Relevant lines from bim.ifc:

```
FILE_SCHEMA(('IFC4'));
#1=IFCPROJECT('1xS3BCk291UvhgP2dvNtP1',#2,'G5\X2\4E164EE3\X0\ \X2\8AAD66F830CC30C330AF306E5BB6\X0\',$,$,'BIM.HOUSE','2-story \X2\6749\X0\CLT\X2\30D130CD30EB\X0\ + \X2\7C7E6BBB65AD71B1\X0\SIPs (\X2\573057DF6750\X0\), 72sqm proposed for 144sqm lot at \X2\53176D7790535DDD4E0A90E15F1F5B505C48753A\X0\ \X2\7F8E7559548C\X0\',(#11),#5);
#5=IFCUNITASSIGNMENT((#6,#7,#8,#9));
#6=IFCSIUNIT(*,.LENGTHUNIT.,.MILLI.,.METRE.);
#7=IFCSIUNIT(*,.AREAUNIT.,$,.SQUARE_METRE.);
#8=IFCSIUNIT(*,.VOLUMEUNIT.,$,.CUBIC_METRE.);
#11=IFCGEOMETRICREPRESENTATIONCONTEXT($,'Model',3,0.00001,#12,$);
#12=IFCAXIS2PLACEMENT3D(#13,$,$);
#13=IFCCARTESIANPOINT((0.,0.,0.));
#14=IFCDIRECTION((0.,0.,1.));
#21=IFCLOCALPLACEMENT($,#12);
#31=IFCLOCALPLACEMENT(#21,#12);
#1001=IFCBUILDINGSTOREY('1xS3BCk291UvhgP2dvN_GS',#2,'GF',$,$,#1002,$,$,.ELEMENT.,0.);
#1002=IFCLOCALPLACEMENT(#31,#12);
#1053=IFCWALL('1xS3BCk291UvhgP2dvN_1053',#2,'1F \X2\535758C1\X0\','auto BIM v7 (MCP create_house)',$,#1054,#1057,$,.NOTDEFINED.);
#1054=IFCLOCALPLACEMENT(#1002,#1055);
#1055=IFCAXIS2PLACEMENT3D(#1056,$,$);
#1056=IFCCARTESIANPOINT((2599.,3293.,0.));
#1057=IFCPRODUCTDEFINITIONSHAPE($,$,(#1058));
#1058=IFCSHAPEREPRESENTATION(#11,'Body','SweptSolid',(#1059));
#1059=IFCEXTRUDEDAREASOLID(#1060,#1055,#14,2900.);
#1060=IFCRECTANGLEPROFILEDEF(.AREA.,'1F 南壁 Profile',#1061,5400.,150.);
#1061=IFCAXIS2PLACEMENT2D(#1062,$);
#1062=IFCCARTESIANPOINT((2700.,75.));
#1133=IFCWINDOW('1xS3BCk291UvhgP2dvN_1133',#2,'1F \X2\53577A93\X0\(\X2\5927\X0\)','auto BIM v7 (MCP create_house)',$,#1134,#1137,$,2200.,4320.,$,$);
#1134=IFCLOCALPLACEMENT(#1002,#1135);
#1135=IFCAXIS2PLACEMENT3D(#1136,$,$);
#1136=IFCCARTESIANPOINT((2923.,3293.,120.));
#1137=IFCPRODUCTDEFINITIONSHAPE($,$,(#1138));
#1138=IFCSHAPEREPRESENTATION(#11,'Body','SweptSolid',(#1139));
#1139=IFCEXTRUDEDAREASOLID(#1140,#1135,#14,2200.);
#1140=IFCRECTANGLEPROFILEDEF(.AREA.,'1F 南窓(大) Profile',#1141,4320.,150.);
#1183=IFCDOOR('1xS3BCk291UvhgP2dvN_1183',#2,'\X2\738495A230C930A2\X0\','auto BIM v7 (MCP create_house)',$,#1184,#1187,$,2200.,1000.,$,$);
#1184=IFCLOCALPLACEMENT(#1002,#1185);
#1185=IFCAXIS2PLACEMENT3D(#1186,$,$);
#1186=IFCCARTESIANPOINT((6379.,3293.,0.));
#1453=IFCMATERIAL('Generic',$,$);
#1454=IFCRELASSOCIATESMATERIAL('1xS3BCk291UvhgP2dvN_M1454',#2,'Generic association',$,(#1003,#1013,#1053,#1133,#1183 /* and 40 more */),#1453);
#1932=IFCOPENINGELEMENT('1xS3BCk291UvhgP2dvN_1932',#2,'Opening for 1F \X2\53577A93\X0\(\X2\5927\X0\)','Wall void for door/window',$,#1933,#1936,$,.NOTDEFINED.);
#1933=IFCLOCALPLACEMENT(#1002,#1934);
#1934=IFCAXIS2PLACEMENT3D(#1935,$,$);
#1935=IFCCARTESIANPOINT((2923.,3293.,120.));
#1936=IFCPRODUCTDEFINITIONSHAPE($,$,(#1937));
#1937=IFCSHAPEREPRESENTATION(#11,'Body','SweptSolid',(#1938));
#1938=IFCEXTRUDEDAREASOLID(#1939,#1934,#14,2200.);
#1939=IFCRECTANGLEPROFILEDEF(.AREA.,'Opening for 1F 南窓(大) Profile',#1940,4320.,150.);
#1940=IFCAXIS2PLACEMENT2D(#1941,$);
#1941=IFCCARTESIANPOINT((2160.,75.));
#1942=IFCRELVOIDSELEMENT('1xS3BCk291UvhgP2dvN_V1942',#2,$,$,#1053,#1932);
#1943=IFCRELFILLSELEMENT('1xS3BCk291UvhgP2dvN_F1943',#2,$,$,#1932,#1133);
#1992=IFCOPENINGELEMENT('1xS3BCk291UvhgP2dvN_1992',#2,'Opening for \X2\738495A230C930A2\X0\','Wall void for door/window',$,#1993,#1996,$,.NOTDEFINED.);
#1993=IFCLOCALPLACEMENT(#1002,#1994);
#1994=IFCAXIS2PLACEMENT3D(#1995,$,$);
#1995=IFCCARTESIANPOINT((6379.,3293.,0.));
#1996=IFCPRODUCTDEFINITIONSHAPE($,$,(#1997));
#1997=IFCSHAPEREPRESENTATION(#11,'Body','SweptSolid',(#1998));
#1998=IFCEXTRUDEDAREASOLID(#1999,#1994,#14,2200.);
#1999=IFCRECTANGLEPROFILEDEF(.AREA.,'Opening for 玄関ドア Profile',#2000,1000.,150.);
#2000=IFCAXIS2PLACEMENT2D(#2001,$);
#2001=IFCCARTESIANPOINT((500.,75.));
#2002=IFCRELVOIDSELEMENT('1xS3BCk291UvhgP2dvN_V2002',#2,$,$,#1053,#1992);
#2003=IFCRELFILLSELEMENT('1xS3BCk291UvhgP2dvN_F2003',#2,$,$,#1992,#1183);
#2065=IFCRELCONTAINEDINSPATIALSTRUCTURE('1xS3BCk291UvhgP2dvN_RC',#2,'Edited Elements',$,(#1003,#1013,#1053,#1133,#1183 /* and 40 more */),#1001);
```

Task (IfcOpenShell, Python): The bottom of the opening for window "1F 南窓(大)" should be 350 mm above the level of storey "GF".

```python
import numpy as np
import ifcopenshell
import ifcopenshell.api.geometry
import ifcopenshell.geom
import ifcopenshell.util.element
import ifcopenshell.util.placement
import ifcopenshell.util.shape
import ifcopenshell.util.unit

model = ifcopenshell.open("bim.ifc")
unit_scale = ifcopenshell.util.unit.calculate_unit_scale(model)

window = model.by_guid("1xS3BCk291UvhgP2dvN_1133")
opening = window.FillsVoids[0].RelatingOpeningElement
storey = ifcopenshell.util.element.get_container(window, ifc_class="IfcBuildingStorey")
level = ifcopenshell.util.placement.get_local_placement(storey.ObjectPlacement)[2, 3]

# The opening's origin need not be at the sill, so measure its lowest point.
shape = ifcopenshell.geom.create_shape(ifcopenshell.geom.settings(), opening)
bottom = ifcopenshell.util.shape.get_shape_bottom_elevation(shape, shape.geometry) / unit_scale
dz = level + 0.35 / unit_scale - bottom

shift = np.array([0.0, 0.0, dz])
# The window is not placed relative to its opening, so move both.
for product in (opening, window):
    matrix = ifcopenshell.util.placement.get_local_placement(product.ObjectPlacement)
    matrix[:3, 3] += shift
    ifcopenshell.api.geometry.edit_object_placement(model, product=product, matrix=matrix, is_si=False)

print(f"moved by {dz * unit_scale:+.3f} m")

model.write("bim_edited.ifc")
```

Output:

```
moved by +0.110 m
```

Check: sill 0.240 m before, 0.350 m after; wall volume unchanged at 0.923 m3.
